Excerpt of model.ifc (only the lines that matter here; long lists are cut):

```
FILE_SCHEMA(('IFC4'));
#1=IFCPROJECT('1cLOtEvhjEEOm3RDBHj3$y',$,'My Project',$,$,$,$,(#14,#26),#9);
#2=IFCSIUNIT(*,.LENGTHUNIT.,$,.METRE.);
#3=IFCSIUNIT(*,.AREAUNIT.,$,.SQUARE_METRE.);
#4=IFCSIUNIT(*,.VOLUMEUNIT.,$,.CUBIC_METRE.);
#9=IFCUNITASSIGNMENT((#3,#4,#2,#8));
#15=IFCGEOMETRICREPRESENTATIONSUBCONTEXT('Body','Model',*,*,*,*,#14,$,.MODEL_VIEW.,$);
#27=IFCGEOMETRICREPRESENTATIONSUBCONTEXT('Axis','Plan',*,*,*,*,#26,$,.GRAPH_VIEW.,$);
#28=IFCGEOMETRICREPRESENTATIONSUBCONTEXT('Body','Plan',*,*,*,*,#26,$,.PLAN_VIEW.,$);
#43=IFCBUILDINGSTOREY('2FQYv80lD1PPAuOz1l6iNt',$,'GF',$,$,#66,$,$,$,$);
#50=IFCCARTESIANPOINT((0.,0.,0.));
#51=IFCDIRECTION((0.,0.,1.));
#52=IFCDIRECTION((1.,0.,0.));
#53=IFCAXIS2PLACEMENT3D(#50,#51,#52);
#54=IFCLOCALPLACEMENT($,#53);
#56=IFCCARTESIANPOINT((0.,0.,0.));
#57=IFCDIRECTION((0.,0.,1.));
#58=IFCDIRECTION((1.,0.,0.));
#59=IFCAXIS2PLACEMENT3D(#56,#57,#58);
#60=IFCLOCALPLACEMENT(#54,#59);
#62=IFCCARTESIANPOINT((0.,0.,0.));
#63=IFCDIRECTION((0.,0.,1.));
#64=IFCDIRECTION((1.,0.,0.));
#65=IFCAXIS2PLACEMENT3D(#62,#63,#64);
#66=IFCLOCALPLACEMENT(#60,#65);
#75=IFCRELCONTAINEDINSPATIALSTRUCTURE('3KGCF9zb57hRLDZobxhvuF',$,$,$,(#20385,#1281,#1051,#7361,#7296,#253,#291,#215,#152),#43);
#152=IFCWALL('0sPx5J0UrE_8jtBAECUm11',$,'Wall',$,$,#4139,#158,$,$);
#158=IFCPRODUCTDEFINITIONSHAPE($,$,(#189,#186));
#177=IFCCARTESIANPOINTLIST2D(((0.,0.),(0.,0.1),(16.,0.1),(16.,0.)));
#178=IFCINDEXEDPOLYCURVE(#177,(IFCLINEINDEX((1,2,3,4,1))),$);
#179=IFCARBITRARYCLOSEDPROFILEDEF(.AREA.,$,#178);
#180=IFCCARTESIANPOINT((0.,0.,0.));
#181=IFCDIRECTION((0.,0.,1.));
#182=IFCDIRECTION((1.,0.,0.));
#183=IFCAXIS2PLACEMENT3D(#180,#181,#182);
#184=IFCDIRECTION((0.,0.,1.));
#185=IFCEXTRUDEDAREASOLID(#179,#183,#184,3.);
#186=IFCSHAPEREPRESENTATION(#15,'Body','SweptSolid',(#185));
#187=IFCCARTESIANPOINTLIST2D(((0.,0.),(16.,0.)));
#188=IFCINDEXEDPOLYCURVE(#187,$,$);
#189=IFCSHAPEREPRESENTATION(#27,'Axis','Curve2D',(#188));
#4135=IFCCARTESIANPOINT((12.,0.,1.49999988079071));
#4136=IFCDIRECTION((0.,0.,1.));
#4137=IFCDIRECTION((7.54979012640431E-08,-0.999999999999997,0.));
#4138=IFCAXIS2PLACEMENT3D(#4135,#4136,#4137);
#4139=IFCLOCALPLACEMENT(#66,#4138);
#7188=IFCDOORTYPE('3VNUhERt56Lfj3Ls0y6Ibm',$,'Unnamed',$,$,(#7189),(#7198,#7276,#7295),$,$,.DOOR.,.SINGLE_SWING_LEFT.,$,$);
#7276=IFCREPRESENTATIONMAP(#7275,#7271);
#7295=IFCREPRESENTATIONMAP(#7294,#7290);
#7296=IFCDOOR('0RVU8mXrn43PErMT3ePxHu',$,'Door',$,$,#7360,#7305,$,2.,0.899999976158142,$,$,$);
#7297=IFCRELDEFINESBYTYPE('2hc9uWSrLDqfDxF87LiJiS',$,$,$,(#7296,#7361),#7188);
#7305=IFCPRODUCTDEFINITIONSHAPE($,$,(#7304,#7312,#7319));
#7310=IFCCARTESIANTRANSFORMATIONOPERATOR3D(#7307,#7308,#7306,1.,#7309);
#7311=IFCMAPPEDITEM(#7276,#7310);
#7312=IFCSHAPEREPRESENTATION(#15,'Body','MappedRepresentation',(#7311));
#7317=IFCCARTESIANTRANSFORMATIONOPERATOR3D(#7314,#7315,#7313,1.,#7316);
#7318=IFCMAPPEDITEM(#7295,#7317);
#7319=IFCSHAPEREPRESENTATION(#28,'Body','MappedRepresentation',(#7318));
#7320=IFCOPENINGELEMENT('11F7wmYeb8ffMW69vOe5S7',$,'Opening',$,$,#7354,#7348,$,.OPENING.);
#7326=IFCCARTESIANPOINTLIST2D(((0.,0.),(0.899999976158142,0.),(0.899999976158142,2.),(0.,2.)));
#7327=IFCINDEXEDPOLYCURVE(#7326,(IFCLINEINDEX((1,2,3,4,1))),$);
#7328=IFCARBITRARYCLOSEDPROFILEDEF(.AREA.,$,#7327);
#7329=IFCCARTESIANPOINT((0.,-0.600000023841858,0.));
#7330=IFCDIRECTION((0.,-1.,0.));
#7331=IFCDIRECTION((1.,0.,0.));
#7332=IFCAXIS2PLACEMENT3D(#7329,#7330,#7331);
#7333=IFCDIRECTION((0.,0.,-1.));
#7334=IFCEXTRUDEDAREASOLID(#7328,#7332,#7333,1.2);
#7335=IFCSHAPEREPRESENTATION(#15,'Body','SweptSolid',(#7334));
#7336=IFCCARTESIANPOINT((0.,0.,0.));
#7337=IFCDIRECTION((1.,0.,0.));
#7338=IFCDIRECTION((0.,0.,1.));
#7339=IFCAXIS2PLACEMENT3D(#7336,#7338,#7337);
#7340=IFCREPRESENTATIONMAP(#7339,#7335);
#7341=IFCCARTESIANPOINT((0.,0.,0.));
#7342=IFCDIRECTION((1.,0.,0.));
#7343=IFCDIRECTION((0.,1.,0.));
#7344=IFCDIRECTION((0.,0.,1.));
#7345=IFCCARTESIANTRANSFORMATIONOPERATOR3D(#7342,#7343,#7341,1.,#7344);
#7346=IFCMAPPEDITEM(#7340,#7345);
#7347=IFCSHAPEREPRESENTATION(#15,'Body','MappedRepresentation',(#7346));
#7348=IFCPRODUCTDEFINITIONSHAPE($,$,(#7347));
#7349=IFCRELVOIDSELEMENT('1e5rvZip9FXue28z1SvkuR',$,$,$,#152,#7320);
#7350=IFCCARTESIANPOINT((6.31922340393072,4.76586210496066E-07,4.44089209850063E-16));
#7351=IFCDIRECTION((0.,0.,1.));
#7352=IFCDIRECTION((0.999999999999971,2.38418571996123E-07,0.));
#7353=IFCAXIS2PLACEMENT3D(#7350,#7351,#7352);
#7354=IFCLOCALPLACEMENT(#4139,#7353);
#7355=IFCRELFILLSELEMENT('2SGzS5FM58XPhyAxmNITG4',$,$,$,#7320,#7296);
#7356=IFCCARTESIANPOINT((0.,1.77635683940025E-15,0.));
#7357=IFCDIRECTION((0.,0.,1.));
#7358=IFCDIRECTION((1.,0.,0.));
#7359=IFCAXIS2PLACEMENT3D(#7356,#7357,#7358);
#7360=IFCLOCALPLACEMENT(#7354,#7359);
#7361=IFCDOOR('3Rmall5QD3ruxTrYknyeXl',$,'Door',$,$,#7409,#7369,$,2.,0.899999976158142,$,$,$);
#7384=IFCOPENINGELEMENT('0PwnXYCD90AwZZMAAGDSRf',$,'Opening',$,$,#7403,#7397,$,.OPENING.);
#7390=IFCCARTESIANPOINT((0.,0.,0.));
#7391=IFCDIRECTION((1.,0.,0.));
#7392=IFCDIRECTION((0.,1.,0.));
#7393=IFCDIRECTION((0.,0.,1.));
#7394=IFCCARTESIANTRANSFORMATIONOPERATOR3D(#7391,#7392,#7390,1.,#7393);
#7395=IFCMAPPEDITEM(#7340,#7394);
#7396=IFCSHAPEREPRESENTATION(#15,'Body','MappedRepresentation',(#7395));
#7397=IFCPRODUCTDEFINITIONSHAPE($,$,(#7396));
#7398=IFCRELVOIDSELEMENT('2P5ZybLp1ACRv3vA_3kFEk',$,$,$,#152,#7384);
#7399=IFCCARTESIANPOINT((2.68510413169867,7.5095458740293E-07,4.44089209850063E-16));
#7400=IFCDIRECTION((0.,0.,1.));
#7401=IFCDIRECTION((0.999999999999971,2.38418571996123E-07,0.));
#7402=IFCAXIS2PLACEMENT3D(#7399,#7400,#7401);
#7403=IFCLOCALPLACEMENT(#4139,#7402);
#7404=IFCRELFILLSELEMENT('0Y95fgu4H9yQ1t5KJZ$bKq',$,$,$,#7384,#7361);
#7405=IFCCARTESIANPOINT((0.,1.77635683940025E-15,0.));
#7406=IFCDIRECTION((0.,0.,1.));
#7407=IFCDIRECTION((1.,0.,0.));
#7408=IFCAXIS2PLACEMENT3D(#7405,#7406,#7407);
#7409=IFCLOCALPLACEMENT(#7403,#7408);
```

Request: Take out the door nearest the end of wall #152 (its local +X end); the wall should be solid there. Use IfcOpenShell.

```python
import ifcopenshell
import ifcopenshell.api.feature
import ifcopenshell.api.root
import ifcopenshell.geom
import ifcopenshell.util.shape

model = ifcopenshell.open("model.ifc")
settings = ifcopenshell.geom.settings()


def volume(element):
    """Net volume in cubic metres, openings subtracted."""
    shape = ifcopenshell.geom.create_shape(settings, element)
    return ifcopenshell.util.shape.get_volume(shape.geometry)


door = model.by_id(7296)
opening = door.FillsVoids[0].RelatingOpeningElement
wall = opening.VoidsElements[0].RelatingBuildingElement
before = volume(wall)

ifcopenshell.api.root.remove_product(model, product=door)
ifcopenshell.api.feature.remove_feature(model, feature=opening)

after = volume(wall)

print(f"wall volume {before:.3f} -> {after:.3f} m3")

model.write("model_updated.ifc")
```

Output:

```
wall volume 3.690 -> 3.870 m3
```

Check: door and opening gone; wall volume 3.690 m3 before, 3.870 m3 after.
